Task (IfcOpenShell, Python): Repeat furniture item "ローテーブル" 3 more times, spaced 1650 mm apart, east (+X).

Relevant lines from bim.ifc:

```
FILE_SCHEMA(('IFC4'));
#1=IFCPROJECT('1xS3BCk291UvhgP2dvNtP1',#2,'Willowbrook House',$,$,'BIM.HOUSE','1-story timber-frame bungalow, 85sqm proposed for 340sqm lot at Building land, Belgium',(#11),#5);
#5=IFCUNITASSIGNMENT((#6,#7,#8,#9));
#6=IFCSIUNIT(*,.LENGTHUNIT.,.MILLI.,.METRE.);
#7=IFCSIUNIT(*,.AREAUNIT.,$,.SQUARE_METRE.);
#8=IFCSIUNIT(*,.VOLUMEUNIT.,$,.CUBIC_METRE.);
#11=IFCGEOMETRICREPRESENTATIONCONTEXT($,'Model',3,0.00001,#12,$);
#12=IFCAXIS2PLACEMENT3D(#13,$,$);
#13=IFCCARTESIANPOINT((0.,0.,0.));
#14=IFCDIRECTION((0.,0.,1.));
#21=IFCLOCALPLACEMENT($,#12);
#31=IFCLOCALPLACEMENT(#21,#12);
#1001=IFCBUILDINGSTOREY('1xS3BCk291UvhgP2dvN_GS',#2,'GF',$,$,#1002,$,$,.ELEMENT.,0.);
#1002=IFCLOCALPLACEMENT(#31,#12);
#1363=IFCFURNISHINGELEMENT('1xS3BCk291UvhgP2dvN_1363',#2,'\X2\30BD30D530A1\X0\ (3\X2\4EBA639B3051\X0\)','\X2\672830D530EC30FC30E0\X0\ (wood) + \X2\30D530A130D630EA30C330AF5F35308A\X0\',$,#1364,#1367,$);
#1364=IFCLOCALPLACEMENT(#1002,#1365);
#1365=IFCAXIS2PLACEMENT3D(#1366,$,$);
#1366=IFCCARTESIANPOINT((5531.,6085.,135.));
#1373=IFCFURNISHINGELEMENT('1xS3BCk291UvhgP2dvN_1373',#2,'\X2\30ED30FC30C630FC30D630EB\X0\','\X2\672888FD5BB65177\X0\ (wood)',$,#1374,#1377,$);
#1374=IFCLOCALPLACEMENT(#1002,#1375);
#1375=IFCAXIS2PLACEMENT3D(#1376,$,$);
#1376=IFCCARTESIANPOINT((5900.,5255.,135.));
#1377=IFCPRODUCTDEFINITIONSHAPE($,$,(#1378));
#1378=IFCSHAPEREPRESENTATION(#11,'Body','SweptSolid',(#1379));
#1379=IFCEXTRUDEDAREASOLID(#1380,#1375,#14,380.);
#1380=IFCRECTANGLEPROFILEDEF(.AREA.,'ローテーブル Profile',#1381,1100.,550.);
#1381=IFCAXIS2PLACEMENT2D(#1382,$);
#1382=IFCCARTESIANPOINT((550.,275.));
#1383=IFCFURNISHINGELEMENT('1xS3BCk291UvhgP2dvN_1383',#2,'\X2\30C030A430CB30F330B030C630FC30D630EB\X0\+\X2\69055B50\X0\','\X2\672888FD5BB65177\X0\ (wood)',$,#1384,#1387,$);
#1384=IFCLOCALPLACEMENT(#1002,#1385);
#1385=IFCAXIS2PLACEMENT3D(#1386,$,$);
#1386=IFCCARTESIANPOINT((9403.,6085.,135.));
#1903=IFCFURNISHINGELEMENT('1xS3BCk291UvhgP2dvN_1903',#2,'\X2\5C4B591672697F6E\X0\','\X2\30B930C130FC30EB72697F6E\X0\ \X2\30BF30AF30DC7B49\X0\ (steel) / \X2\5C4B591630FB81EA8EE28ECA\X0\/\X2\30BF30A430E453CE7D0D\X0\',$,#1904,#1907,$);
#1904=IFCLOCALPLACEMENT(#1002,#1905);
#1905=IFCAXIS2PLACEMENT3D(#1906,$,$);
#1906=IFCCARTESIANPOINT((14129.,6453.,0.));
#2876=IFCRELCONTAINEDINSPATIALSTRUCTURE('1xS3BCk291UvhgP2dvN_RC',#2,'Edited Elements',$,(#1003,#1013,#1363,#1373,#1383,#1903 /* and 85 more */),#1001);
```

```python
import numpy as np
import ifcopenshell
import ifcopenshell.api.geometry
import ifcopenshell.api.root
import ifcopenshell.util.element
import ifcopenshell.util.placement

model = ifcopenshell.open("bim.ifc")


def reuse_history(source, copy):
    """copy_class also copies each property set's owner history, people and application; keep the originals."""
    for rel in copy.IsDefinedBy:
        if rel.is_a("IfcRelDefinesByProperties") and (history := rel.RelatingPropertyDefinition.OwnerHistory):
            rel.RelatingPropertyDefinition.OwnerHistory = source.OwnerHistory
            ifcopenshell.util.element.remove_deep2(model, history)


source = model.by_guid("1xS3BCk291UvhgP2dvN_1373")
base = ifcopenshell.util.placement.get_local_placement(source.ObjectPlacement)
step = np.array([1.0, 0.0, 0.0]) * 1650.0

for i in range(1, 4):
    copy = ifcopenshell.api.root.copy_class(model, product=source)
    copy.Representation = ifcopenshell.util.element.copy_deep(
        model, source.Representation, exclude=["IfcGeometricRepresentationContext", "IfcRepresentationMap"]
    )
    reuse_history(source, copy)
    matrix = base.copy()
    matrix[:3, 3] += i * step
    print("added at", matrix[:3, 3].round(3) + 0.0)
    ifcopenshell.api.geometry.edit_object_placement(model, product=copy, matrix=matrix, is_si=False)

model.write("bim-out.ifc")
```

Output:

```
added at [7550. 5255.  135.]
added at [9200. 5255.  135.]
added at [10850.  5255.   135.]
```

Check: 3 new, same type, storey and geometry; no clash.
